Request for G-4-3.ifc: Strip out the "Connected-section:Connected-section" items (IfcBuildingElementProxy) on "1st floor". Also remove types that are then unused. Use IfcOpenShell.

First a look at what the model holds.

```python
import ifcopenshell
import ifcopenshell.util.element

model = ifcopenshell.open("G-4-3.ifc")
print(model.schema)
storey = next(s for s in model.by_type("IfcBuildingStorey") if s.Name == "1st floor")
proxies = [e for e in ifcopenshell.util.element.get_decomposition(storey) if e.is_a("IfcBuildingElementProxy")]
seen = {}
for e in proxies:
    element_type = ifcopenshell.util.element.get_type(e)
    name = element_type.Name if element_type not in (None, e) else None
    seen[name] = seen.get(name, 0) + 1
for name, count in sorted(seen.items(), key=str):
    print(count, "x", name)
```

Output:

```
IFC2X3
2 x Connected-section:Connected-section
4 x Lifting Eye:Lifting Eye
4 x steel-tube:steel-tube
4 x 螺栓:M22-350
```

```python
import ifcopenshell
import ifcopenshell.api.root
import ifcopenshell.util.element

model = ifcopenshell.open("G-4-3.ifc")

storey = next(s for s in model.by_type("IfcBuildingStorey") if s.Name == "1st floor")
proxies = [e for e in ifcopenshell.util.element.get_decomposition(storey) if e.is_a("IfcBuildingElementProxy")]
targets = [e for e in proxies if (t := ifcopenshell.util.element.get_type(e)) not in (None, e) and t.Name == "Connected-section:Connected-section"]
types = {ifcopenshell.util.element.get_type(e) for e in targets} - {None, *targets}

for e in targets:
    ifcopenshell.api.root.remove_product(model, product=e)
print(len(targets), "removed")

unused = [t for t in types if not ifcopenshell.util.element.get_types(t)]
for t in unused:
    ifcopenshell.api.root.remove_product(model, product=t)
print(len(unused), "unused types removed")

model.write("G-4-3_rev.ifc")
```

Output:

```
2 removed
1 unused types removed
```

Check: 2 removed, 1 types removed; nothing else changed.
